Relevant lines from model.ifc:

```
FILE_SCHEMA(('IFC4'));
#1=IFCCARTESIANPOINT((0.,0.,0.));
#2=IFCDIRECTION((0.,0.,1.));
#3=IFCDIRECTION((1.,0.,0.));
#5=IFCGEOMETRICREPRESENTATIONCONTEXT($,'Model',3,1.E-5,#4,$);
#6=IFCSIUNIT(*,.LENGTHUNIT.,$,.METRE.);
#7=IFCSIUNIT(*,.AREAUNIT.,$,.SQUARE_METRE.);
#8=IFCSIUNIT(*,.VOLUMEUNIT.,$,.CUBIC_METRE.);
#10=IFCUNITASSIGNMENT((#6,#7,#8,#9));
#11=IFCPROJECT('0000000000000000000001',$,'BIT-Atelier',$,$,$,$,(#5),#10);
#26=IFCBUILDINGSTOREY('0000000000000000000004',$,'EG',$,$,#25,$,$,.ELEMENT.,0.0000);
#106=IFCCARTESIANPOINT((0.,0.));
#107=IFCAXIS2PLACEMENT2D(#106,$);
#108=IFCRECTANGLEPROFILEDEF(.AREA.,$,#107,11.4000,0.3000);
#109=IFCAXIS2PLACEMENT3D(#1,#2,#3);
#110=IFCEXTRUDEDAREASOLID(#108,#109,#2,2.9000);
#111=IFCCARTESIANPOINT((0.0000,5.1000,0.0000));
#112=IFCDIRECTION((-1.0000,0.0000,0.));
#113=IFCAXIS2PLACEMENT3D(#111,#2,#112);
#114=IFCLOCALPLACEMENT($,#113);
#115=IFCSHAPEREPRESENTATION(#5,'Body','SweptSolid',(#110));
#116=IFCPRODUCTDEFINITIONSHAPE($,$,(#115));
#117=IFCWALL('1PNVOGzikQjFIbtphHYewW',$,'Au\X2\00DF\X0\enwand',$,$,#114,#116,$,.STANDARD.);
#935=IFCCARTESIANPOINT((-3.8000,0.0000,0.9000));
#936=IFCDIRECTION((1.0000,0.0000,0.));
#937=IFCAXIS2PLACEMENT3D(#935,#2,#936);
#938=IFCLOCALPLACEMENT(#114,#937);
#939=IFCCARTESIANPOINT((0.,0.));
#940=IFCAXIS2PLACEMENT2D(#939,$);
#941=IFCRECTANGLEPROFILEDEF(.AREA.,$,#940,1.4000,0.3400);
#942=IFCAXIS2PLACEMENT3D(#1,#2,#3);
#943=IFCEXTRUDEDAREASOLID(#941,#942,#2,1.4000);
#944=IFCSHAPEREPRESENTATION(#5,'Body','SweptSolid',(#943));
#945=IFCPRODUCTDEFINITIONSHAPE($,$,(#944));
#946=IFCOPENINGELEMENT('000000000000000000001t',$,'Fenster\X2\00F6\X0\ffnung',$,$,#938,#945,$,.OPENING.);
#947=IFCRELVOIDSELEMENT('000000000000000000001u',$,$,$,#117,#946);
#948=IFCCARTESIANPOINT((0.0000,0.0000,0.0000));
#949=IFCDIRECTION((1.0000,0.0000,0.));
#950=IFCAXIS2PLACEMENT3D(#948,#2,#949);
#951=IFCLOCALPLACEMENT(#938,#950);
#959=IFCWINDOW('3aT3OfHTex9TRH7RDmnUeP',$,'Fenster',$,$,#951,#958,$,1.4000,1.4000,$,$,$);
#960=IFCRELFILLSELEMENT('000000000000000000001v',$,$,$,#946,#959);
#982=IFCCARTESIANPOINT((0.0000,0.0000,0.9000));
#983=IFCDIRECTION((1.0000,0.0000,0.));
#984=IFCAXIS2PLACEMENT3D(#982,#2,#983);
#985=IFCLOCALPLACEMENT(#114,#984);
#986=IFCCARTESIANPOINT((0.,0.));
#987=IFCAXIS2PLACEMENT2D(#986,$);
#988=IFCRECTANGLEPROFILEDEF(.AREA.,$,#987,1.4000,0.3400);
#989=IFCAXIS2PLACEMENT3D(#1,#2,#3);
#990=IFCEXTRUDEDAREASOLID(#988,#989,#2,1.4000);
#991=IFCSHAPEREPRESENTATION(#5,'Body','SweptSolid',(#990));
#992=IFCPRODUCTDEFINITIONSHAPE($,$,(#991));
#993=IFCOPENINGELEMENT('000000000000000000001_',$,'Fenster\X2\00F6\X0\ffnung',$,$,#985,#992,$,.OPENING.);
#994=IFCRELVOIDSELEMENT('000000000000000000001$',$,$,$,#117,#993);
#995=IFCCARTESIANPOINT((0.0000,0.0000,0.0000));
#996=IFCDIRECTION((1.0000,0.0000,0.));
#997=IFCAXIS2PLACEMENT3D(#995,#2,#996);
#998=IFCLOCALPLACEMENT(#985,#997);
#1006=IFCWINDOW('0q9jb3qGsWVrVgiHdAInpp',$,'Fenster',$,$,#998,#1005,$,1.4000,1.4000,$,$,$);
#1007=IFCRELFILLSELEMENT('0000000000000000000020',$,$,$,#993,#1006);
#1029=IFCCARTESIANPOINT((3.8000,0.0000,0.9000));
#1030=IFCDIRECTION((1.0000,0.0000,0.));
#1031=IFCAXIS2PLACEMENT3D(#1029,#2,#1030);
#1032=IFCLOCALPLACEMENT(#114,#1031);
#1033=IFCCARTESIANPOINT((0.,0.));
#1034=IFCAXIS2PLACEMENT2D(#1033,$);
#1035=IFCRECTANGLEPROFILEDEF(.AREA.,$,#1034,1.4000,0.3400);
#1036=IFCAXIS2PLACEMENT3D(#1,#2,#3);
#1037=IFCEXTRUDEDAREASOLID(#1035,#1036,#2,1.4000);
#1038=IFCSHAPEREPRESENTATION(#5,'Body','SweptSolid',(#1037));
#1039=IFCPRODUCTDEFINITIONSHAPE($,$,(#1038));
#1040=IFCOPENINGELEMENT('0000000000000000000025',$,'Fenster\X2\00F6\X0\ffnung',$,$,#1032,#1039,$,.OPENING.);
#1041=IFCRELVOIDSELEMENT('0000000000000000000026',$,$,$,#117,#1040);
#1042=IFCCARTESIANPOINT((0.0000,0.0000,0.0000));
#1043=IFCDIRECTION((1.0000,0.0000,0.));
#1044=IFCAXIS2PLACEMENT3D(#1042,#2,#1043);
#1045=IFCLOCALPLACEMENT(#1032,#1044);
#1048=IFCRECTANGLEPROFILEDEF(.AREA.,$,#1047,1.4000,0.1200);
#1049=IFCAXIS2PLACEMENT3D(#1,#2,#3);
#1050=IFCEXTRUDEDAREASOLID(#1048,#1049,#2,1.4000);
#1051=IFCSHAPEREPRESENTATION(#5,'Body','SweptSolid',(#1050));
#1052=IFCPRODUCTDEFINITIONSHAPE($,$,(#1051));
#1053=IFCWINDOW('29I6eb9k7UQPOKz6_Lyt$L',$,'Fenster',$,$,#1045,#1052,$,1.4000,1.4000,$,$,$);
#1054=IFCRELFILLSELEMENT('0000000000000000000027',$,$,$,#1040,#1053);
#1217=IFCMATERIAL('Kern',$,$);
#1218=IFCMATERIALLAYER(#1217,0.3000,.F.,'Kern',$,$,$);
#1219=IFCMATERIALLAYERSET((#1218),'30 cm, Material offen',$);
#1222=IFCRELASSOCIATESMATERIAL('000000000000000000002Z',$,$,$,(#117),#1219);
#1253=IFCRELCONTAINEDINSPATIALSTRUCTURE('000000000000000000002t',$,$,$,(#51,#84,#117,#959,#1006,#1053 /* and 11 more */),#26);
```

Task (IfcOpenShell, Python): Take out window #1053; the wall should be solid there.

```python
import ifcopenshell
import ifcopenshell.api.feature
import ifcopenshell.api.root
import ifcopenshell.geom
import ifcopenshell.util.shape

model = ifcopenshell.open("model.ifc")
settings = ifcopenshell.geom.settings()


def volume(element):
    """Net volume in cubic metres, openings subtracted."""
    shape = ifcopenshell.geom.create_shape(settings, element)
    return ifcopenshell.util.shape.get_volume(shape.geometry)


window = model.by_id(1053)
opening = window.FillsVoids[0].RelatingOpeningElement
wall = opening.VoidsElements[0].RelatingBuildingElement
before = volume(wall)

ifcopenshell.api.root.remove_product(model, product=window)
ifcopenshell.api.feature.remove_feature(model, feature=opening)

after = volume(wall)

print(f"wall volume {before:.3f} -> {after:.3f} m3")

model.write("model_updated.ifc")
```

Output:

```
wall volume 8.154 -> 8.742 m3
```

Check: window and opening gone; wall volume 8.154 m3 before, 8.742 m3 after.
